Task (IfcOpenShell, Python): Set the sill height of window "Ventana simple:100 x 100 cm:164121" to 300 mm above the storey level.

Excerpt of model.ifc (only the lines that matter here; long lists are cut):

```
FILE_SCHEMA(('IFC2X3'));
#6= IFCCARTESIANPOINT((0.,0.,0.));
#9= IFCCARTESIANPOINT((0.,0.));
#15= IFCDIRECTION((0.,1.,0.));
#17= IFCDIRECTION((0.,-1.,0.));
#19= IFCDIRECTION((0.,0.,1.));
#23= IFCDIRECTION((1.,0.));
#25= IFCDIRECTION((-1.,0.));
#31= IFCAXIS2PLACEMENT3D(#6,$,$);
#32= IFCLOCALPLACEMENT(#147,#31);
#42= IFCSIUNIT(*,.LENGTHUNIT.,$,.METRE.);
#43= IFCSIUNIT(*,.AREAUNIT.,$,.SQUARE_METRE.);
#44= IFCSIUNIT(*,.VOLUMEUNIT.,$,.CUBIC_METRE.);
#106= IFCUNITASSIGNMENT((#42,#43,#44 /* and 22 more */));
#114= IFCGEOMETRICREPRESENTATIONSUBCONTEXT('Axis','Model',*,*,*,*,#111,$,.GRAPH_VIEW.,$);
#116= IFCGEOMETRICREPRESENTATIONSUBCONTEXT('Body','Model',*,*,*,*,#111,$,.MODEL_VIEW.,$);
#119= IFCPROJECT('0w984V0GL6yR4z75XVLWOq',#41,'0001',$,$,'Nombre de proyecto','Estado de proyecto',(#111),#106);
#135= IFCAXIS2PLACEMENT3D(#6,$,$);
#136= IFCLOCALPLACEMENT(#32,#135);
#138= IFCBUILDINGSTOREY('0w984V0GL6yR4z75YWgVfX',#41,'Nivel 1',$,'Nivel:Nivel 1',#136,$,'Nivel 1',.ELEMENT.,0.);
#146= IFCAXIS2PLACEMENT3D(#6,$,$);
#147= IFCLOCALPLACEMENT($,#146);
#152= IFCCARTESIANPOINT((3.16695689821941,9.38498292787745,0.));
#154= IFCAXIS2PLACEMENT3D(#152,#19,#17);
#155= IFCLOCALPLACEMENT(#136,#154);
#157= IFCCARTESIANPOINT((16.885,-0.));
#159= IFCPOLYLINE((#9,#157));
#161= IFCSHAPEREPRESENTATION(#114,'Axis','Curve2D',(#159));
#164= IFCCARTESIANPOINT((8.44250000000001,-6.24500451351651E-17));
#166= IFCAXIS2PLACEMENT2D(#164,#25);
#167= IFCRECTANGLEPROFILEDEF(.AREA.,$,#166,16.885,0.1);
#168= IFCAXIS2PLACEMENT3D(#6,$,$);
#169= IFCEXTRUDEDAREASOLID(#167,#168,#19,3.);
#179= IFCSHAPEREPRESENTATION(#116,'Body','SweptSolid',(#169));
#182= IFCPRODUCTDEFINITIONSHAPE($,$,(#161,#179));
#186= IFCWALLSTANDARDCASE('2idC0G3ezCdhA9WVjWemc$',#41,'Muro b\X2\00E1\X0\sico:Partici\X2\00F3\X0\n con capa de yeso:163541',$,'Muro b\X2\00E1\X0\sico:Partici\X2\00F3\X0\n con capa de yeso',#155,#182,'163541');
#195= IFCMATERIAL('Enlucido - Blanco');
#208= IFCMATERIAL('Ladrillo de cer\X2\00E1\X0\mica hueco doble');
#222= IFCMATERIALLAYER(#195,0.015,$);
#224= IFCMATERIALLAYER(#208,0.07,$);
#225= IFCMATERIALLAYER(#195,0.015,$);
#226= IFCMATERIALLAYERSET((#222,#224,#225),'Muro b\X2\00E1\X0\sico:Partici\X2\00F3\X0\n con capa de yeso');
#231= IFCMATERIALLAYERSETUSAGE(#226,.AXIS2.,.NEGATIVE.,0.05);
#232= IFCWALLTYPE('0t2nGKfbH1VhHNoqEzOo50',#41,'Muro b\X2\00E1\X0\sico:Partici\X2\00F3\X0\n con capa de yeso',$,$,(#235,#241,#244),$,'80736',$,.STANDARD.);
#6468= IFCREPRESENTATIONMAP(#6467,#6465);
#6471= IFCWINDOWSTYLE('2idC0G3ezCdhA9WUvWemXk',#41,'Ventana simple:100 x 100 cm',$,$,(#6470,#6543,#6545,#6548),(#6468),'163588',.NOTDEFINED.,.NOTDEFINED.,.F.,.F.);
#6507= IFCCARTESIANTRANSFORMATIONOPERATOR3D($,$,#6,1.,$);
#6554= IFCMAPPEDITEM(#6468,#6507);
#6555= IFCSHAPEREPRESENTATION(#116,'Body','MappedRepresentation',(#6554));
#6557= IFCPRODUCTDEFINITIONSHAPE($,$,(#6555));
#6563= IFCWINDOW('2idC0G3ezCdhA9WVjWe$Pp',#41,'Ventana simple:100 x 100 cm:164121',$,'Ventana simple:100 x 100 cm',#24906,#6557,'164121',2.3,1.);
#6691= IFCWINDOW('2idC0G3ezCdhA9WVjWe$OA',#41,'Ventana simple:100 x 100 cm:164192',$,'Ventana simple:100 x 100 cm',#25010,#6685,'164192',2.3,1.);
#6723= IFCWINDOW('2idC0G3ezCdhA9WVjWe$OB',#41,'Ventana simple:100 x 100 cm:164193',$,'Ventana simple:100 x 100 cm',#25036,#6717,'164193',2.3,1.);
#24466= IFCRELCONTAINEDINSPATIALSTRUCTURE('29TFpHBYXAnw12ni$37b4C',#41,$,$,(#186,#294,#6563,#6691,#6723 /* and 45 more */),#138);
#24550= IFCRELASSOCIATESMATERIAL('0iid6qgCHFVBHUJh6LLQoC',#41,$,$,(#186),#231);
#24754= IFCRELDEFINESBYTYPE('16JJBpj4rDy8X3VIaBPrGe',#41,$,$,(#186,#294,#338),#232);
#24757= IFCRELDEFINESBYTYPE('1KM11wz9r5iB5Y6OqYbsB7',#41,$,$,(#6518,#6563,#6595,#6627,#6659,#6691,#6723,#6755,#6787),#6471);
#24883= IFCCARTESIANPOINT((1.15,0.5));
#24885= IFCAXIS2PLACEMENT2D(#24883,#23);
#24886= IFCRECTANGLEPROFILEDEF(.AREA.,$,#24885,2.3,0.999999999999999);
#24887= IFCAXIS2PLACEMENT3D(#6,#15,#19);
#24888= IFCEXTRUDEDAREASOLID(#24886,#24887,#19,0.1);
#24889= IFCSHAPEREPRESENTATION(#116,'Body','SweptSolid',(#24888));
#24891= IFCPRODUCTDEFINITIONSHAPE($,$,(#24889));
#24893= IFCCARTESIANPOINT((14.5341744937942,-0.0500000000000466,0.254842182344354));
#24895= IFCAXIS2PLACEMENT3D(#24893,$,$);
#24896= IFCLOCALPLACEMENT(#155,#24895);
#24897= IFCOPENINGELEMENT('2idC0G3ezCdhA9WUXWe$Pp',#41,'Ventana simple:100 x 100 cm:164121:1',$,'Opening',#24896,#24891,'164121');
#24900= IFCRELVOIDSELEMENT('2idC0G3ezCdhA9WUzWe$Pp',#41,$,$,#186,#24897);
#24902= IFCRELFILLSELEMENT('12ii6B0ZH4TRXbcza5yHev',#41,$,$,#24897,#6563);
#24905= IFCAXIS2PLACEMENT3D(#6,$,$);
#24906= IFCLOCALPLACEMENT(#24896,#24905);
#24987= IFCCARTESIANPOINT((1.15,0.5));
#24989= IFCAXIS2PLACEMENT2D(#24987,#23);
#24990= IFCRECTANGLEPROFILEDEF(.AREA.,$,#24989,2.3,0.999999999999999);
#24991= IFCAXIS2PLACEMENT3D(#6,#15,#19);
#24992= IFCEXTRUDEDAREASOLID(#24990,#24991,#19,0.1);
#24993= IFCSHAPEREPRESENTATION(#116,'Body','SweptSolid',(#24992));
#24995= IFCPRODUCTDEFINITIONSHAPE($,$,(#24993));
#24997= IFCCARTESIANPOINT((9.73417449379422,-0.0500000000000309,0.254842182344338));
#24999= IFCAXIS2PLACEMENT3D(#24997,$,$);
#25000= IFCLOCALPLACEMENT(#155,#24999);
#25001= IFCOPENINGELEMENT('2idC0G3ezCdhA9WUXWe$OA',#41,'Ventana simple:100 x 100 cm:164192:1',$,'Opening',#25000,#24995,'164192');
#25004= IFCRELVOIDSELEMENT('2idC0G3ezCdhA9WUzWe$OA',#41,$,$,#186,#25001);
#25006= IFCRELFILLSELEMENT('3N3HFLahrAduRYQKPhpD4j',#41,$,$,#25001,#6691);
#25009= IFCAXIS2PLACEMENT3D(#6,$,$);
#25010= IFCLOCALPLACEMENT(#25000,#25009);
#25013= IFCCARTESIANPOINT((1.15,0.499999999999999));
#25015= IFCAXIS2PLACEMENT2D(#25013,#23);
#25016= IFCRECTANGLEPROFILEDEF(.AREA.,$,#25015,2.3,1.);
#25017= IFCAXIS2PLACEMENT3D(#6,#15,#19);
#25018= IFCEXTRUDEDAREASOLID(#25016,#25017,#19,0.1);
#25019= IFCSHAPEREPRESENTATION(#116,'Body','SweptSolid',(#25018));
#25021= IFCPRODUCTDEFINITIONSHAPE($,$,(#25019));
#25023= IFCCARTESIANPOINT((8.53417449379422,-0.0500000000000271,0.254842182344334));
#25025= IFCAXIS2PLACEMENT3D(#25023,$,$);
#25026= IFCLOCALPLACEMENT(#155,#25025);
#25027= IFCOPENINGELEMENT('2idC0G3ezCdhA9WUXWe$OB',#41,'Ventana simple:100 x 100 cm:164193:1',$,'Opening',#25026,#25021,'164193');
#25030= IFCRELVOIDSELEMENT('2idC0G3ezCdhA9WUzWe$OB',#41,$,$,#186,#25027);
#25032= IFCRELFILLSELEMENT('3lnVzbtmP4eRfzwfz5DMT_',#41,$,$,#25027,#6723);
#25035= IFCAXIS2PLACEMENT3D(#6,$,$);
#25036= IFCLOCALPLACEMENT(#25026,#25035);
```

```python
import numpy as np
import ifcopenshell
import ifcopenshell.api.geometry
import ifcopenshell.geom
import ifcopenshell.util.element
import ifcopenshell.util.placement
import ifcopenshell.util.shape
import ifcopenshell.util.unit

model = ifcopenshell.open("model.ifc")
unit_scale = ifcopenshell.util.unit.calculate_unit_scale(model)

window = model.by_guid("2idC0G3ezCdhA9WVjWe$Pp")
opening = window.FillsVoids[0].RelatingOpeningElement
storey = ifcopenshell.util.element.get_container(window, ifc_class="IfcBuildingStorey")
level = ifcopenshell.util.placement.get_local_placement(storey.ObjectPlacement)[2, 3]

# The opening's origin need not be at the sill, so measure its lowest point.
shape = ifcopenshell.geom.create_shape(ifcopenshell.geom.settings(), opening)
bottom = ifcopenshell.util.shape.get_shape_bottom_elevation(shape, shape.geometry) / unit_scale
dz = level + 0.3 / unit_scale - bottom

shift = np.array([0.0, 0.0, dz])
# The window is placed relative to its opening, so it follows when the opening moves.
matrix = ifcopenshell.util.placement.get_local_placement(opening.ObjectPlacement)
matrix[:3, 3] += shift
ifcopenshell.api.geometry.edit_object_placement(
    model, product=opening, matrix=matrix, is_si=False, should_transform_children=True
)

print(f"moved by {dz * unit_scale:+.3f} m")

model.write("model_v2.ifc")
```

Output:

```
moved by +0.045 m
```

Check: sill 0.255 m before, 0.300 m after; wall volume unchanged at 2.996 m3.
